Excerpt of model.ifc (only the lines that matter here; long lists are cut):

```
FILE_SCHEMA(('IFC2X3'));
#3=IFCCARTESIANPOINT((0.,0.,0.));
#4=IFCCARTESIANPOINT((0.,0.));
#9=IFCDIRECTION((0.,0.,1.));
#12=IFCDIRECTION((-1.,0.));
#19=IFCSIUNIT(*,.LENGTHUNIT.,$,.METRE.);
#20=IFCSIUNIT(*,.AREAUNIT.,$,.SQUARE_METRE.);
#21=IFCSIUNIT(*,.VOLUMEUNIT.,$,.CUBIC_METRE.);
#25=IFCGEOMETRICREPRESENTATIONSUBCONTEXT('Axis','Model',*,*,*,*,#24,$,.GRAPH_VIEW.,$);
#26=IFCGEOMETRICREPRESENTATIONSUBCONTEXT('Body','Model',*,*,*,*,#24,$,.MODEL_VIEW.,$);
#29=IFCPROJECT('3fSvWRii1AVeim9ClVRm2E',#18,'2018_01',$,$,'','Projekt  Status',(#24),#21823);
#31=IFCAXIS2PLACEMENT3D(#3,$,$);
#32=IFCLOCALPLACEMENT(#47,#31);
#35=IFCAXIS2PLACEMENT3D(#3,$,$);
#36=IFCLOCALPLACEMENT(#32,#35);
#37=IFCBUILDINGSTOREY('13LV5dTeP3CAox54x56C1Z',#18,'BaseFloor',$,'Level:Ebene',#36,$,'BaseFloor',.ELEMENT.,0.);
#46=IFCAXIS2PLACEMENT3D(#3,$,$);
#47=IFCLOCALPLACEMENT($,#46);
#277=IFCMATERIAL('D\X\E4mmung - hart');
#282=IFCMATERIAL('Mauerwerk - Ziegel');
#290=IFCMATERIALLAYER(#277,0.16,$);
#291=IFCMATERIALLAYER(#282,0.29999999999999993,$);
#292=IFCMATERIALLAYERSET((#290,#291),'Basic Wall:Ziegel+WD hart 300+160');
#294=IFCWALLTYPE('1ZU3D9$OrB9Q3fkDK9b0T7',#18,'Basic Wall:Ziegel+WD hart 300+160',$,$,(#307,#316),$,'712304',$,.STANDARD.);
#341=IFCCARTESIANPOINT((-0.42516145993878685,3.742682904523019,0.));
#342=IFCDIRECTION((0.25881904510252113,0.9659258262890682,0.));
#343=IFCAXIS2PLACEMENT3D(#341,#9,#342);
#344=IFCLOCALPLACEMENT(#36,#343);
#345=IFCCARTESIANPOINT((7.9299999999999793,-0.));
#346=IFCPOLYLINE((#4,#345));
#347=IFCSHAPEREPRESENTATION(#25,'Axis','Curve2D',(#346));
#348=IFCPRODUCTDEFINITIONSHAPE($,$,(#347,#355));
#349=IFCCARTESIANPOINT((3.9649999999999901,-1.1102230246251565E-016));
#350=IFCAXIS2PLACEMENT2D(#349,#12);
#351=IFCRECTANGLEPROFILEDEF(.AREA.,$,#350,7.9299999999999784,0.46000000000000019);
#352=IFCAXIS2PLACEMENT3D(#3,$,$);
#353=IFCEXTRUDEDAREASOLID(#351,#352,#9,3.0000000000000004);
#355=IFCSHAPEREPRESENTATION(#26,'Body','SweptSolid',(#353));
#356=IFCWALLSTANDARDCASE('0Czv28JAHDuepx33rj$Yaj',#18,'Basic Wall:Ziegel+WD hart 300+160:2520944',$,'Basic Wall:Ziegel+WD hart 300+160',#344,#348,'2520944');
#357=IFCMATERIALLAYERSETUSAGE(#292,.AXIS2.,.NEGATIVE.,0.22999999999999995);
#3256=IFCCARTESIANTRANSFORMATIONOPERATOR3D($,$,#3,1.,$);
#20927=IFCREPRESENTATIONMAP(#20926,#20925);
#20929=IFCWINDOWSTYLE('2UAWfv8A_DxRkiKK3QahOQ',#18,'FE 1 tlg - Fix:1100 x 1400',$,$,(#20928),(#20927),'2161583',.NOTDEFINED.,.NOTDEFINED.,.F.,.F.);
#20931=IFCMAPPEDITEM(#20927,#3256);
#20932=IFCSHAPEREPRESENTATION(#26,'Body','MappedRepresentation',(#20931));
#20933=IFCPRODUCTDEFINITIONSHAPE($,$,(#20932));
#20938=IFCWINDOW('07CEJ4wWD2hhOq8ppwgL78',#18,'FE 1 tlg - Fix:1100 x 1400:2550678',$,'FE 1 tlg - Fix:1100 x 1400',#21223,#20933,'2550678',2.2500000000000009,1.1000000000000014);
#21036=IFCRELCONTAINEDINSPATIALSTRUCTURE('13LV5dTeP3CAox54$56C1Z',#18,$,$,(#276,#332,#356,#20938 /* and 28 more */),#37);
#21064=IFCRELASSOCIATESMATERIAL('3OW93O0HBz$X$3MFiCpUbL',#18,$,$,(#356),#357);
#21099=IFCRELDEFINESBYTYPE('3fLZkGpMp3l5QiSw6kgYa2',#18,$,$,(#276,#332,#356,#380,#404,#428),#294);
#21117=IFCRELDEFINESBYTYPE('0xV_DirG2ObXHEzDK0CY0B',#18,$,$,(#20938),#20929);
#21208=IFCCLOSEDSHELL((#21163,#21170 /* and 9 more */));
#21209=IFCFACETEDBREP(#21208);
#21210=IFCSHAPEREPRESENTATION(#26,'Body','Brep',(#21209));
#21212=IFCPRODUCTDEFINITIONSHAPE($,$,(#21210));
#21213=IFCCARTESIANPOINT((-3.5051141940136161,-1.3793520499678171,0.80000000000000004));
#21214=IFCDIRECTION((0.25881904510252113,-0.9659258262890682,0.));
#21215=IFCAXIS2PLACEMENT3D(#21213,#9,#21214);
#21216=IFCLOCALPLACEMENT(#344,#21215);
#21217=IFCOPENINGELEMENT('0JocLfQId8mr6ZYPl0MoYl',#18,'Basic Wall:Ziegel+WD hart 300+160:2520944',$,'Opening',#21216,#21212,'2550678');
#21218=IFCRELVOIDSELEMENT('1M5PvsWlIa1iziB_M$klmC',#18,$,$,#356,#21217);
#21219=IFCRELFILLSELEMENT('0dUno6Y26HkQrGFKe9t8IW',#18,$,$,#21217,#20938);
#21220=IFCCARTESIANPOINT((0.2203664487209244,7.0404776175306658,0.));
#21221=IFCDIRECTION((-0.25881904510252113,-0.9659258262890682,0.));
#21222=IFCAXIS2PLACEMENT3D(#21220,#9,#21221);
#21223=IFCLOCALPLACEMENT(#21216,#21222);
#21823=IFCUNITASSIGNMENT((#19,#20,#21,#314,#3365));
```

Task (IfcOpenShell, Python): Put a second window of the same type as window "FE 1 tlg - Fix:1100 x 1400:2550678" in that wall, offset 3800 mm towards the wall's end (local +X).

```python
import ifcopenshell
import ifcopenshell.api.feature
import ifcopenshell.api.geometry
import ifcopenshell.api.root
import ifcopenshell.geom
import ifcopenshell.util.element
import ifcopenshell.util.placement
import ifcopenshell.util.shape
import ifcopenshell.util.unit

model = ifcopenshell.open("model.ifc")
unit_scale = ifcopenshell.util.unit.calculate_unit_scale(model)
settings = ifcopenshell.geom.settings()


def volume(element):
    """Net volume in cubic metres, openings subtracted."""
    shape = ifcopenshell.geom.create_shape(settings, element)
    return ifcopenshell.util.shape.get_volume(shape.geometry)


def reuse_history(source, copy):
    """copy_class also copies each property set's owner history, people and application; keep the originals."""
    for rel in copy.IsDefinedBy:
        if rel.is_a("IfcRelDefinesByProperties") and (history := rel.RelatingPropertyDefinition.OwnerHistory):
            rel.RelatingPropertyDefinition.OwnerHistory = source.OwnerHistory
            ifcopenshell.util.element.remove_deep2(model, history)


window = model.by_id(20938)
opening = window.FillsVoids[0].RelatingOpeningElement
wall = opening.VoidsElements[0].RelatingBuildingElement
before = volume(wall)
shift = ifcopenshell.util.placement.get_local_placement(wall.ObjectPlacement)[:3, 0] * 3.8 / unit_scale

# copy_class copies the void relationship, type, container and properties, but no geometry.
new_opening = ifcopenshell.api.root.copy_class(model, product=opening)
new_opening.Representation = ifcopenshell.util.element.copy_deep(
    model, opening.Representation, exclude=["IfcGeometricRepresentationContext", "IfcRepresentationMap"]
)
new_opening.Name = "Basic Wall:Ziegel+WD hart 300+160"
new_opening.Tag = None
new_window = ifcopenshell.api.root.copy_class(model, product=window)
new_window.Representation = ifcopenshell.util.element.copy_deep(
    model, window.Representation, exclude=["IfcGeometricRepresentationContext", "IfcRepresentationMap"]
)
new_window.Name = "FE 1 tlg - Fix:1100 x 1400"
new_window.Tag = None
reuse_history(window, new_window)
fills = ifcopenshell.api.feature.add_filling(model, opening=new_opening, element=new_window)
fills.OwnerHistory = new_window.OwnerHistory  # required in IFC2X3

for old, new in ((opening, new_opening), (window, new_window)):
    matrix = ifcopenshell.util.placement.get_local_placement(old.ObjectPlacement)
    matrix[:3, 3] += shift
    ifcopenshell.api.geometry.edit_object_placement(model, product=new, matrix=matrix, is_si=False)

after = volume(wall)

print(f"wall volume {before:.3f} -> {after:.3f} m3")

model.write("model_updated.ifc")
```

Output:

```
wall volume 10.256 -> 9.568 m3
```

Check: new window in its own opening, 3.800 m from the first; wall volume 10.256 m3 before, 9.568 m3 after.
